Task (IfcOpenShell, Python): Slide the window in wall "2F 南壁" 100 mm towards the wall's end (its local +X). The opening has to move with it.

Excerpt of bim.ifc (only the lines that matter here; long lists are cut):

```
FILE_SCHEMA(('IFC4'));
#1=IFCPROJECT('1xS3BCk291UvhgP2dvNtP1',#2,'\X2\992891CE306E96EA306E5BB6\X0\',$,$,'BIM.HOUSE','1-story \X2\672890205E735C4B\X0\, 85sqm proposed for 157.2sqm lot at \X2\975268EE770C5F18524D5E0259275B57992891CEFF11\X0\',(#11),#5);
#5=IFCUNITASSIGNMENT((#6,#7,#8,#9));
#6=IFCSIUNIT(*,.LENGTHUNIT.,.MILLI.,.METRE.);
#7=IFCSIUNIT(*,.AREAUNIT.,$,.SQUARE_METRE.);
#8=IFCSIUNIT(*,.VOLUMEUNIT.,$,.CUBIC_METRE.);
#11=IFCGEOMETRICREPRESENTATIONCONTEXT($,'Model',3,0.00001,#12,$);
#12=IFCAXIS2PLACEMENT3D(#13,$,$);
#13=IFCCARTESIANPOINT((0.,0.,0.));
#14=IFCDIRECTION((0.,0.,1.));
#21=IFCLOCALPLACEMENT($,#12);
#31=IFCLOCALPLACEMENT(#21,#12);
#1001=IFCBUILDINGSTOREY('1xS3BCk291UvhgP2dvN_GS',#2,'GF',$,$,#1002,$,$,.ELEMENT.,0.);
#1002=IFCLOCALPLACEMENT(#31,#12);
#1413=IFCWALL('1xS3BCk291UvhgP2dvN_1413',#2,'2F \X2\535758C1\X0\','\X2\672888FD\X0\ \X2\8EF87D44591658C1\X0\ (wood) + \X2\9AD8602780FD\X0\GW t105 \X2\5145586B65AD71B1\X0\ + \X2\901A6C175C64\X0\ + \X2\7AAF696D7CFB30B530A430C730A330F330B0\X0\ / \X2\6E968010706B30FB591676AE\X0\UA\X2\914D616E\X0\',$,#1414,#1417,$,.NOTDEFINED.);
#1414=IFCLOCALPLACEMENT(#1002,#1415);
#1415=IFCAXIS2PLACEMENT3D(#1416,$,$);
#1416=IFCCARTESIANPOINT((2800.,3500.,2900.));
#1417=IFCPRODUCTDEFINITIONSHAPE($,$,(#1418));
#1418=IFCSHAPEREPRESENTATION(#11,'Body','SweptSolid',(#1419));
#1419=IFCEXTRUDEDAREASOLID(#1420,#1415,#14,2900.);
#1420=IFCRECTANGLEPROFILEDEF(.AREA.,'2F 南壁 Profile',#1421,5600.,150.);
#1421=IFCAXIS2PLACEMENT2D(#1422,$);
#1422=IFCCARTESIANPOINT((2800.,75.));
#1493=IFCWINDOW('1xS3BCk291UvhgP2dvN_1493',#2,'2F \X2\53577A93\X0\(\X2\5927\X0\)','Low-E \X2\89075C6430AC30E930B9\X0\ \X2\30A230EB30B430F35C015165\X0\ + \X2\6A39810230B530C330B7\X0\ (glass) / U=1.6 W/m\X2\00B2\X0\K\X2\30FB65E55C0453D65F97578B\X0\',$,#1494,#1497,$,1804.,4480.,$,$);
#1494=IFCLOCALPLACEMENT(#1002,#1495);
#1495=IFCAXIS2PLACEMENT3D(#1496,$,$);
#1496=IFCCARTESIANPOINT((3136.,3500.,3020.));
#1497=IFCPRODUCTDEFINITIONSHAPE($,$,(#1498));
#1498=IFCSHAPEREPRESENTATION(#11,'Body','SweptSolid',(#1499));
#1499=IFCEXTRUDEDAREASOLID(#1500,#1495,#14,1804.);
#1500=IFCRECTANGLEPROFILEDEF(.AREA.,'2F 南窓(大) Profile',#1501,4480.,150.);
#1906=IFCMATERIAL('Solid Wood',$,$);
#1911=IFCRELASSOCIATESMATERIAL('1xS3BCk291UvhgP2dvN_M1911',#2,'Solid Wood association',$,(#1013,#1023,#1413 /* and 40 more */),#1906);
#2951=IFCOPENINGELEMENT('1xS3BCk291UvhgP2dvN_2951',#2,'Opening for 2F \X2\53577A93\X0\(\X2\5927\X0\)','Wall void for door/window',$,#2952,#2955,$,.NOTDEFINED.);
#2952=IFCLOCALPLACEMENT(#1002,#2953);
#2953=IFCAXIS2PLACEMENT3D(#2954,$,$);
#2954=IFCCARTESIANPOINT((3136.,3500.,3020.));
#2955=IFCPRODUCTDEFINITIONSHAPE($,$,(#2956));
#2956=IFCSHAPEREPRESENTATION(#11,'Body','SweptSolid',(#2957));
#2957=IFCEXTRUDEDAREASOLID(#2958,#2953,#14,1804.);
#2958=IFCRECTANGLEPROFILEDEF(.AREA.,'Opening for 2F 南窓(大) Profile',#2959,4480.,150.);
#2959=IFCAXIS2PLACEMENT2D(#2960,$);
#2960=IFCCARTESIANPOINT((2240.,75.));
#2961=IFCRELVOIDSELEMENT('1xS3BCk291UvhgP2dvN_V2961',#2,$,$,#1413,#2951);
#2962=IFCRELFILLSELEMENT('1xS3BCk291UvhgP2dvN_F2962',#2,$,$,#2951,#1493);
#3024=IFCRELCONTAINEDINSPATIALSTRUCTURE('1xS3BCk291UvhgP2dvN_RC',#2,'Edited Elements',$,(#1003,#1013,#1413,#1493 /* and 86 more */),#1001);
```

```python
import ifcopenshell
import ifcopenshell.api.geometry
import ifcopenshell.util.placement
import ifcopenshell.util.unit

model = ifcopenshell.open("bim.ifc")
unit_scale = ifcopenshell.util.unit.calculate_unit_scale(model)

window = model.by_guid("1xS3BCk291UvhgP2dvN_1493")
opening = window.FillsVoids[0].RelatingOpeningElement
wall = opening.VoidsElements[0].RelatingBuildingElement

wall_matrix = ifcopenshell.util.placement.get_local_placement(wall.ObjectPlacement)
shift = wall_matrix[:3, 0] * 0.1 / unit_scale
before = ifcopenshell.util.placement.get_local_placement(window.ObjectPlacement)[:3, 3].copy()

# The window is not placed relative to its opening, so move both.
for product in (opening, window):
    matrix = ifcopenshell.util.placement.get_local_placement(product.ObjectPlacement)
    matrix[:3, 3] += shift
    ifcopenshell.api.geometry.edit_object_placement(model, product=product, matrix=matrix, is_si=False)

after = ifcopenshell.util.placement.get_local_placement(window.ObjectPlacement)[:3, 3]
print("window moved by", (after - before).round(3) + 0.0)

model.write("bim-out.ifc")
```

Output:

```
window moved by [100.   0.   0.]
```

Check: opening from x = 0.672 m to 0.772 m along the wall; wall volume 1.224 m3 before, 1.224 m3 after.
